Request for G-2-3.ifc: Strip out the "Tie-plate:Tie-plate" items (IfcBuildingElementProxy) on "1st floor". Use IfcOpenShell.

First a look at what the model holds.

```python
import ifcopenshell
import ifcopenshell.util.element

model = ifcopenshell.open("G-2-3.ifc")
print(model.schema)
storey = next(s for s in model.by_type("IfcBuildingStorey") if s.Name == "1st floor")
proxies = [e for e in ifcopenshell.util.element.get_decomposition(storey) if e.is_a("IfcBuildingElementProxy")]
seen = {}
for e in proxies:
    element_type = ifcopenshell.util.element.get_type(e)
    name = element_type.Name if element_type not in (None, e) else None
    seen[name] = seen.get(name, 0) + 1
for name, count in sorted(seen.items(), key=str):
    print(count, "x", name)
```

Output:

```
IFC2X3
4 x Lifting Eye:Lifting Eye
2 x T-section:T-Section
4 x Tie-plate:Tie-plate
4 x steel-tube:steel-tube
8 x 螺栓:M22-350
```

```python
import ifcopenshell
import ifcopenshell.api.root
import ifcopenshell.util.element

model = ifcopenshell.open("G-2-3.ifc")

storey = next(s for s in model.by_type("IfcBuildingStorey") if s.Name == "1st floor")
proxies = [e for e in ifcopenshell.util.element.get_decomposition(storey) if e.is_a("IfcBuildingElementProxy")]
targets = [e for e in proxies if (t := ifcopenshell.util.element.get_type(e)) not in (None, e) and t.Name == "Tie-plate:Tie-plate"]

for e in targets:
    ifcopenshell.api.root.remove_product(model, product=e)
print(len(targets), "removed")

model.write("G-2-3_v2.ifc")
```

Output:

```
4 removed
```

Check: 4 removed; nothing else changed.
